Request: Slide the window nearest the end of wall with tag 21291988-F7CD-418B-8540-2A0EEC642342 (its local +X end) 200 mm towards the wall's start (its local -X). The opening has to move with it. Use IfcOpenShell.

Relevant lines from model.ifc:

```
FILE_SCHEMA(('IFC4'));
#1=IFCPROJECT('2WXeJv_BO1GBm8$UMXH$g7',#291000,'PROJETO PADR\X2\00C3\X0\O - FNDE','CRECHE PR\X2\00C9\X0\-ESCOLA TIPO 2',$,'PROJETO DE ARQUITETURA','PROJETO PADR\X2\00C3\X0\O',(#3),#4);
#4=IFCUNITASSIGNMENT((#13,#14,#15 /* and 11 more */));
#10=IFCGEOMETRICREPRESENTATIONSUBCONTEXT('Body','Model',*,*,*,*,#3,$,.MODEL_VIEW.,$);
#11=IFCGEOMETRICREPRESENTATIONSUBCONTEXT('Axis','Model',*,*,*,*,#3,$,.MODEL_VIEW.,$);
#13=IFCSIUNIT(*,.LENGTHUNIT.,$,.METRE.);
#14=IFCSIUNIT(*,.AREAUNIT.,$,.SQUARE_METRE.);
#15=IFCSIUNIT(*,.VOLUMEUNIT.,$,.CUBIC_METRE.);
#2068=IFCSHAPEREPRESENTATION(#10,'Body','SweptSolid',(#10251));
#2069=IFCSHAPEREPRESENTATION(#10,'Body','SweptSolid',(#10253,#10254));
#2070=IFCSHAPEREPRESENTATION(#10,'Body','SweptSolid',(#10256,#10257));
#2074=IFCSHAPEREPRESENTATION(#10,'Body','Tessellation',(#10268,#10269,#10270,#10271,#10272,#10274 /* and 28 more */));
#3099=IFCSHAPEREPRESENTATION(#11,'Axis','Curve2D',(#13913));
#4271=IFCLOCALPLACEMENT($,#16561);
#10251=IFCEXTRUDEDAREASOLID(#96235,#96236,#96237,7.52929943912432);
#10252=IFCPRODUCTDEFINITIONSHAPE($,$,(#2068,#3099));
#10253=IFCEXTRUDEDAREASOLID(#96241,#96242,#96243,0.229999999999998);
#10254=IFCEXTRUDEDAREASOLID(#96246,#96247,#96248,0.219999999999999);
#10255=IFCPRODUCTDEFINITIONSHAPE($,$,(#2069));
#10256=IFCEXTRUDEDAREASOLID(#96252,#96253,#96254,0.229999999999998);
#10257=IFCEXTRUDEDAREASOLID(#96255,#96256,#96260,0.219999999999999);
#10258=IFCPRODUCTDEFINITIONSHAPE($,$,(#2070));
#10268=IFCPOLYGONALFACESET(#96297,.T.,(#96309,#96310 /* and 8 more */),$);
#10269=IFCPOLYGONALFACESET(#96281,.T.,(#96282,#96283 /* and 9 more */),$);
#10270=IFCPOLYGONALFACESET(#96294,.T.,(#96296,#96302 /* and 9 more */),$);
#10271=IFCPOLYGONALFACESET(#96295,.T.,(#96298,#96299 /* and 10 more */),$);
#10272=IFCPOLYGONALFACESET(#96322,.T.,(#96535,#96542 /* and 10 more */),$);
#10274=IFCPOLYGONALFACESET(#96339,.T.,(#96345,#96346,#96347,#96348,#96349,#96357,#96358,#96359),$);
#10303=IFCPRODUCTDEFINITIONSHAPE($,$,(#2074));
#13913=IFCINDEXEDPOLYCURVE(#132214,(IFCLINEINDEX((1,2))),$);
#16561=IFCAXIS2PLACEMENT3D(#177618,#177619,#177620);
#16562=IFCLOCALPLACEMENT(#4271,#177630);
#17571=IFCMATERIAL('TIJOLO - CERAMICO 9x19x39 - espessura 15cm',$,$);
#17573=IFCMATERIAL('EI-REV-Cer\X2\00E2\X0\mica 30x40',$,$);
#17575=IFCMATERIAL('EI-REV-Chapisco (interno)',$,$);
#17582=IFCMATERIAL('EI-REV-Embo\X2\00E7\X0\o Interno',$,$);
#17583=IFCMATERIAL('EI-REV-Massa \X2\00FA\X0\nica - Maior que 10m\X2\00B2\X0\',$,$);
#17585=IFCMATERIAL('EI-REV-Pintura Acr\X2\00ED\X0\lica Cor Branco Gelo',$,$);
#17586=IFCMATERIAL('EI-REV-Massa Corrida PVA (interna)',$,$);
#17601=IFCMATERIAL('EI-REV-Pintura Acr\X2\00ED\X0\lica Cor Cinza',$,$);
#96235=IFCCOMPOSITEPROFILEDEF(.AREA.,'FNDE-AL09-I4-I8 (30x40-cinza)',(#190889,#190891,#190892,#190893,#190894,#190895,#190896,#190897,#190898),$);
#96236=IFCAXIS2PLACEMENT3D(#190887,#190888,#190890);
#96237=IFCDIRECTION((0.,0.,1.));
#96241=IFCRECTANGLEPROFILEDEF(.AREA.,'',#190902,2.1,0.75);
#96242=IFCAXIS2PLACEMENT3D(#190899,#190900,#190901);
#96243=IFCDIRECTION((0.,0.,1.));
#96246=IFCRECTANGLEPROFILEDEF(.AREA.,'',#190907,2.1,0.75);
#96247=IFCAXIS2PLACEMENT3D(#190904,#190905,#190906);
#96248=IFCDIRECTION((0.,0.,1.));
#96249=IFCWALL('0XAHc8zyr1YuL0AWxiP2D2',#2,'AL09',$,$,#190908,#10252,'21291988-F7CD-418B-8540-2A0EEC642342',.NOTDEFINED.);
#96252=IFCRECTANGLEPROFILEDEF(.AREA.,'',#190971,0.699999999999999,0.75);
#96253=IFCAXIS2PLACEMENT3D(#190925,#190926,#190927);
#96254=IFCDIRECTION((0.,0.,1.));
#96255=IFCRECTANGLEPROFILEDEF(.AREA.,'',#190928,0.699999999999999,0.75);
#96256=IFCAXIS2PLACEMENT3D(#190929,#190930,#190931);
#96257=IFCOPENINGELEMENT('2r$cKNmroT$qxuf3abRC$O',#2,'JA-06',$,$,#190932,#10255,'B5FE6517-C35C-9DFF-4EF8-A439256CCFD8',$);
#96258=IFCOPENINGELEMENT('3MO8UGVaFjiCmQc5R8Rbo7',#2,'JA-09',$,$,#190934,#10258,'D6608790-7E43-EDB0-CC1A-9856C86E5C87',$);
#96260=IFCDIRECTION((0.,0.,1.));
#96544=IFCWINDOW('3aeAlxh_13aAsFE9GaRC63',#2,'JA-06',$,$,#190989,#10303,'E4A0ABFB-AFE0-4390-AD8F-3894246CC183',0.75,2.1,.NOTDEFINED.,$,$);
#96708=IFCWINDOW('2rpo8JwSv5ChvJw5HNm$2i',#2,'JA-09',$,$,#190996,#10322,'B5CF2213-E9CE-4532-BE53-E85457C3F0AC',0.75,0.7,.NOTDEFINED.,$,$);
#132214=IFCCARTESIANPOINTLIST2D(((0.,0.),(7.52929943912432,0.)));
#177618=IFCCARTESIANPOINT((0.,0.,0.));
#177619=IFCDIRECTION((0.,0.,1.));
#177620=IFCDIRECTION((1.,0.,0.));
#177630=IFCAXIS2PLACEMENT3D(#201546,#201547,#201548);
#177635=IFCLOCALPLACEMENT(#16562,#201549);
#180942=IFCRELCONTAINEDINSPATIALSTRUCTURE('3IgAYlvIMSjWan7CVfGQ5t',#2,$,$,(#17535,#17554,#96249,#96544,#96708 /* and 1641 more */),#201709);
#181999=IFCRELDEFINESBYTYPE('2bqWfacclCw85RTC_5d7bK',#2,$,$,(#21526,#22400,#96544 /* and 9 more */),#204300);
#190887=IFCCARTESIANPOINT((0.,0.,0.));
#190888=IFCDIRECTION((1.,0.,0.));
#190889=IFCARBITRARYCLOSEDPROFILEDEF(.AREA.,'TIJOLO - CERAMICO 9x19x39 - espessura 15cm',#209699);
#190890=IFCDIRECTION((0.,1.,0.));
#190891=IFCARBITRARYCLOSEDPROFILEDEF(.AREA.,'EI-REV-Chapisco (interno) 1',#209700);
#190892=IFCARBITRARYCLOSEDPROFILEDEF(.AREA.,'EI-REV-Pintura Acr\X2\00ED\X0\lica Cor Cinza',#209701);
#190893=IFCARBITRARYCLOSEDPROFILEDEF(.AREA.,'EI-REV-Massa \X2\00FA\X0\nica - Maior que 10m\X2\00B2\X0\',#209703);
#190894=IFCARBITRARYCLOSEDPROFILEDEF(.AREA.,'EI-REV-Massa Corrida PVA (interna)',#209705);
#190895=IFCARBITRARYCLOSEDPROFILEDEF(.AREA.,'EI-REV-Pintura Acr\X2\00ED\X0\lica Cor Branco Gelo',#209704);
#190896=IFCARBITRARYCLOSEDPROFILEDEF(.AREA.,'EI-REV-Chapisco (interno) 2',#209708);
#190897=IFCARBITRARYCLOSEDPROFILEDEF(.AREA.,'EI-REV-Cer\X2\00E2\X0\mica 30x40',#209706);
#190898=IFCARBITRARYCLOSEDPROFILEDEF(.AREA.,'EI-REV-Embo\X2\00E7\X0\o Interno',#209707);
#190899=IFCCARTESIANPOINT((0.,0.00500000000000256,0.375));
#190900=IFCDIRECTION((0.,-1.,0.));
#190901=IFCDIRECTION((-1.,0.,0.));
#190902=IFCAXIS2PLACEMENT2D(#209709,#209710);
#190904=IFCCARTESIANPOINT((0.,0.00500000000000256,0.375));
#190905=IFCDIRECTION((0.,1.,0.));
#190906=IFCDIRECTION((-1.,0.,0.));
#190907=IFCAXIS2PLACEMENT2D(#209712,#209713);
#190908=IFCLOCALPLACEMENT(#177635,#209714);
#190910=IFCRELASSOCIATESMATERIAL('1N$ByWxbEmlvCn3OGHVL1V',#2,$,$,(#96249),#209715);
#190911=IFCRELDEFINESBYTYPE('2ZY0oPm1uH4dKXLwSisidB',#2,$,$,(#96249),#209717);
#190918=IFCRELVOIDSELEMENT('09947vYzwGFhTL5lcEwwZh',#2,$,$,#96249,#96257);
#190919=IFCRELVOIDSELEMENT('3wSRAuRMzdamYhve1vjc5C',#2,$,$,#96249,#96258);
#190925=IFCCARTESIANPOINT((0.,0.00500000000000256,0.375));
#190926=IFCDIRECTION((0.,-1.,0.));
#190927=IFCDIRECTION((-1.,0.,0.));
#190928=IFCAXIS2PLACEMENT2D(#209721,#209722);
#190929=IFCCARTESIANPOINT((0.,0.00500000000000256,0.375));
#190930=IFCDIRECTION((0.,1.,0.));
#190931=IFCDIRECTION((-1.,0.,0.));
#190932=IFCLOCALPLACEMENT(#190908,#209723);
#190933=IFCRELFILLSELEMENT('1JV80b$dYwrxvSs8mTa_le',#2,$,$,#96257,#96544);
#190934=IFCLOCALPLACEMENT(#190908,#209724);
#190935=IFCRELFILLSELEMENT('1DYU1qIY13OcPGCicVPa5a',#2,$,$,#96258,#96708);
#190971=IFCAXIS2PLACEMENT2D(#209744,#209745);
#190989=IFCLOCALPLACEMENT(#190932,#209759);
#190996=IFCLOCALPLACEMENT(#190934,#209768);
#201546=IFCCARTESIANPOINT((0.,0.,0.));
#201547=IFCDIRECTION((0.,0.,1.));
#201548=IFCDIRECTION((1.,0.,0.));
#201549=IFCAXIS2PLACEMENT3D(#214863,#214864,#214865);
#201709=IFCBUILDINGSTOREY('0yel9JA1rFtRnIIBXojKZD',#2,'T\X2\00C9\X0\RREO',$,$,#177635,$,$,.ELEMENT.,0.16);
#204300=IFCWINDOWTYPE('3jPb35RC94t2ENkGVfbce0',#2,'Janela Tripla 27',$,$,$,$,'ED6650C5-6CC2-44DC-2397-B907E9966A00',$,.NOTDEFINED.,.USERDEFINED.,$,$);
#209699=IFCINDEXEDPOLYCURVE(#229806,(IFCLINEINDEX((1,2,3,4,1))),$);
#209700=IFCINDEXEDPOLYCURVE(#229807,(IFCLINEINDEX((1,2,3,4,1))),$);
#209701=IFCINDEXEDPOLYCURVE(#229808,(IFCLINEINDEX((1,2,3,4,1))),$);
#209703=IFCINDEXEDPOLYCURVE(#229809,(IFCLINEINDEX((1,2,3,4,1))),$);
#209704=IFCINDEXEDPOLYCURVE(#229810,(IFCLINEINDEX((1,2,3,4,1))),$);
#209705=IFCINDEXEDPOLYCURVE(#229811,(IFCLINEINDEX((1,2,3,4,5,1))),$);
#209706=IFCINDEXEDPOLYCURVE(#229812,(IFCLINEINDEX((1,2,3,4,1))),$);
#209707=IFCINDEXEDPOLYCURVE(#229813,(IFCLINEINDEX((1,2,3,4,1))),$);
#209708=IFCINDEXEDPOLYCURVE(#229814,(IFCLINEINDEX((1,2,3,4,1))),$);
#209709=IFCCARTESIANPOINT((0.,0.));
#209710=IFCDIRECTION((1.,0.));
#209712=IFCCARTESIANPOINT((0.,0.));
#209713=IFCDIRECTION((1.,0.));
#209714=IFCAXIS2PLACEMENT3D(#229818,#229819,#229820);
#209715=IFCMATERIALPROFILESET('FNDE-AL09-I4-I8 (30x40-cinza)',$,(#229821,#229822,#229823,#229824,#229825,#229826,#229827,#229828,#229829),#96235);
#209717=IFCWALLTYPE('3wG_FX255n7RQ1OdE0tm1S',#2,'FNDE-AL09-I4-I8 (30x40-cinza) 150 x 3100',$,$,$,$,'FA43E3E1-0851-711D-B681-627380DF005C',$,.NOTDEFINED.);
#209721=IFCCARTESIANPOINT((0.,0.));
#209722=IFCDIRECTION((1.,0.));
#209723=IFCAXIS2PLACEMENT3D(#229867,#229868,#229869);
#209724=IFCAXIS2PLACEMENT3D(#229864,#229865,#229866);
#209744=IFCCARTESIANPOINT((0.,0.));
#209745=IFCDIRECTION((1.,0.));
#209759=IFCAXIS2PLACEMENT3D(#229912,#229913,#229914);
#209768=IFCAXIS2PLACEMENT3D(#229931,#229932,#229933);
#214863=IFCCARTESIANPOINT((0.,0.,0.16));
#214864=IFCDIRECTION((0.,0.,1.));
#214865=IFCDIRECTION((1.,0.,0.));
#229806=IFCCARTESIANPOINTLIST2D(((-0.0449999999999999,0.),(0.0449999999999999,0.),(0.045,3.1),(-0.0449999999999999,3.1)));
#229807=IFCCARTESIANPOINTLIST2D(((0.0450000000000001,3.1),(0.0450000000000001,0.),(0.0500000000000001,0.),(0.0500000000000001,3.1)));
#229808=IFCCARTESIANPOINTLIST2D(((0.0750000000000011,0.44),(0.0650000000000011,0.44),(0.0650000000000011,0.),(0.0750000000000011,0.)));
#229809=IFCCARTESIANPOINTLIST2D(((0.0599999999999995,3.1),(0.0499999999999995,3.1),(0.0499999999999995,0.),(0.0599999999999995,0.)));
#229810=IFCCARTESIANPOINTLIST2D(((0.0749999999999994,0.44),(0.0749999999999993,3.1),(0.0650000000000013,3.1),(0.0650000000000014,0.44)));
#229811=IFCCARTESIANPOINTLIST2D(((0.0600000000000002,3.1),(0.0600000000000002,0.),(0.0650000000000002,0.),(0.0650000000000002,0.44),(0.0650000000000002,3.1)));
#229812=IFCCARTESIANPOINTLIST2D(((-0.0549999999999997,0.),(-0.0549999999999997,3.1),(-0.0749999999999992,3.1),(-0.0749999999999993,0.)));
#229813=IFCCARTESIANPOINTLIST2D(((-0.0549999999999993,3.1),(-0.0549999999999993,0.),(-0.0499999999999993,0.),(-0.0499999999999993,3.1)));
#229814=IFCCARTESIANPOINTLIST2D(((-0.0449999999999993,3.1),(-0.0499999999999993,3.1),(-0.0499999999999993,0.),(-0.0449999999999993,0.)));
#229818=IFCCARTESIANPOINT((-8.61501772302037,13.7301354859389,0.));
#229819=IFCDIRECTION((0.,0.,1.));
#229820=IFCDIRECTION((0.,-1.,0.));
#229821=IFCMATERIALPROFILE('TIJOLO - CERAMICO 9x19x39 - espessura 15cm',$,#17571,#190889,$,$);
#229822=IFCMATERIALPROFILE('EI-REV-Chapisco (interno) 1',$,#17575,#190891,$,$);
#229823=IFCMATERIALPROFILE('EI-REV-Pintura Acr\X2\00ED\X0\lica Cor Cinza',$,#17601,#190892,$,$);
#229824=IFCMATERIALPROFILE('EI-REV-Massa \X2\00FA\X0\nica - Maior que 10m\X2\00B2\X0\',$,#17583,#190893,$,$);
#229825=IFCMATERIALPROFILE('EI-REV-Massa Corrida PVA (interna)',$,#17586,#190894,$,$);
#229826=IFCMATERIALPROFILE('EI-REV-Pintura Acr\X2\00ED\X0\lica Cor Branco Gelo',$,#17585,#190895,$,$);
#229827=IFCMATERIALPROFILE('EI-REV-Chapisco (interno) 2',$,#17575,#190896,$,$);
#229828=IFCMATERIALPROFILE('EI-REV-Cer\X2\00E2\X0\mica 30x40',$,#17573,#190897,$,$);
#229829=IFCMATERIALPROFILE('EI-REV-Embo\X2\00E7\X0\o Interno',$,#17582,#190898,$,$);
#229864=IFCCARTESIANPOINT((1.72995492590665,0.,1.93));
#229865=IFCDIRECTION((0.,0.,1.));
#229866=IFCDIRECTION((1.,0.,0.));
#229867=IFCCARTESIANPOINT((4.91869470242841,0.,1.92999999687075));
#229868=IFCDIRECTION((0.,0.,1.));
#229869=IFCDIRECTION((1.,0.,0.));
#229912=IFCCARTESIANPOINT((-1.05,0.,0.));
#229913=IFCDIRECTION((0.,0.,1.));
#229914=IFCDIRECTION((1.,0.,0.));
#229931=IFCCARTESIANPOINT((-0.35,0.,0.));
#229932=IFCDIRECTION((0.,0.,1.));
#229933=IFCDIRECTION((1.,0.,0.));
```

```python
import ifcopenshell
import ifcopenshell.api.geometry
import ifcopenshell.util.placement
import ifcopenshell.util.unit

model = ifcopenshell.open("model.ifc")
unit_scale = ifcopenshell.util.unit.calculate_unit_scale(model)

window = model.by_id(96544)
opening = window.FillsVoids[0].RelatingOpeningElement
wall = opening.VoidsElements[0].RelatingBuildingElement

wall_matrix = ifcopenshell.util.placement.get_local_placement(wall.ObjectPlacement)
shift = wall_matrix[:3, 0] * -0.2 / unit_scale
before = ifcopenshell.util.placement.get_local_placement(window.ObjectPlacement)[:3, 3].copy()

# The window is placed relative to its opening, so it follows when the opening moves.
matrix = ifcopenshell.util.placement.get_local_placement(opening.ObjectPlacement)
matrix[:3, 3] += shift
ifcopenshell.api.geometry.edit_object_placement(
    model, product=opening, matrix=matrix, is_si=False, should_transform_children=True
)

after = ifcopenshell.util.placement.get_local_placement(window.ObjectPlacement)[:3, 3]
print("window moved by", (after - before).round(3) + 0.0)

model.write("model_rev.ifc")
```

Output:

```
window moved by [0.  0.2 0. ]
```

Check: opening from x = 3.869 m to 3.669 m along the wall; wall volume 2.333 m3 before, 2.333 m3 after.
